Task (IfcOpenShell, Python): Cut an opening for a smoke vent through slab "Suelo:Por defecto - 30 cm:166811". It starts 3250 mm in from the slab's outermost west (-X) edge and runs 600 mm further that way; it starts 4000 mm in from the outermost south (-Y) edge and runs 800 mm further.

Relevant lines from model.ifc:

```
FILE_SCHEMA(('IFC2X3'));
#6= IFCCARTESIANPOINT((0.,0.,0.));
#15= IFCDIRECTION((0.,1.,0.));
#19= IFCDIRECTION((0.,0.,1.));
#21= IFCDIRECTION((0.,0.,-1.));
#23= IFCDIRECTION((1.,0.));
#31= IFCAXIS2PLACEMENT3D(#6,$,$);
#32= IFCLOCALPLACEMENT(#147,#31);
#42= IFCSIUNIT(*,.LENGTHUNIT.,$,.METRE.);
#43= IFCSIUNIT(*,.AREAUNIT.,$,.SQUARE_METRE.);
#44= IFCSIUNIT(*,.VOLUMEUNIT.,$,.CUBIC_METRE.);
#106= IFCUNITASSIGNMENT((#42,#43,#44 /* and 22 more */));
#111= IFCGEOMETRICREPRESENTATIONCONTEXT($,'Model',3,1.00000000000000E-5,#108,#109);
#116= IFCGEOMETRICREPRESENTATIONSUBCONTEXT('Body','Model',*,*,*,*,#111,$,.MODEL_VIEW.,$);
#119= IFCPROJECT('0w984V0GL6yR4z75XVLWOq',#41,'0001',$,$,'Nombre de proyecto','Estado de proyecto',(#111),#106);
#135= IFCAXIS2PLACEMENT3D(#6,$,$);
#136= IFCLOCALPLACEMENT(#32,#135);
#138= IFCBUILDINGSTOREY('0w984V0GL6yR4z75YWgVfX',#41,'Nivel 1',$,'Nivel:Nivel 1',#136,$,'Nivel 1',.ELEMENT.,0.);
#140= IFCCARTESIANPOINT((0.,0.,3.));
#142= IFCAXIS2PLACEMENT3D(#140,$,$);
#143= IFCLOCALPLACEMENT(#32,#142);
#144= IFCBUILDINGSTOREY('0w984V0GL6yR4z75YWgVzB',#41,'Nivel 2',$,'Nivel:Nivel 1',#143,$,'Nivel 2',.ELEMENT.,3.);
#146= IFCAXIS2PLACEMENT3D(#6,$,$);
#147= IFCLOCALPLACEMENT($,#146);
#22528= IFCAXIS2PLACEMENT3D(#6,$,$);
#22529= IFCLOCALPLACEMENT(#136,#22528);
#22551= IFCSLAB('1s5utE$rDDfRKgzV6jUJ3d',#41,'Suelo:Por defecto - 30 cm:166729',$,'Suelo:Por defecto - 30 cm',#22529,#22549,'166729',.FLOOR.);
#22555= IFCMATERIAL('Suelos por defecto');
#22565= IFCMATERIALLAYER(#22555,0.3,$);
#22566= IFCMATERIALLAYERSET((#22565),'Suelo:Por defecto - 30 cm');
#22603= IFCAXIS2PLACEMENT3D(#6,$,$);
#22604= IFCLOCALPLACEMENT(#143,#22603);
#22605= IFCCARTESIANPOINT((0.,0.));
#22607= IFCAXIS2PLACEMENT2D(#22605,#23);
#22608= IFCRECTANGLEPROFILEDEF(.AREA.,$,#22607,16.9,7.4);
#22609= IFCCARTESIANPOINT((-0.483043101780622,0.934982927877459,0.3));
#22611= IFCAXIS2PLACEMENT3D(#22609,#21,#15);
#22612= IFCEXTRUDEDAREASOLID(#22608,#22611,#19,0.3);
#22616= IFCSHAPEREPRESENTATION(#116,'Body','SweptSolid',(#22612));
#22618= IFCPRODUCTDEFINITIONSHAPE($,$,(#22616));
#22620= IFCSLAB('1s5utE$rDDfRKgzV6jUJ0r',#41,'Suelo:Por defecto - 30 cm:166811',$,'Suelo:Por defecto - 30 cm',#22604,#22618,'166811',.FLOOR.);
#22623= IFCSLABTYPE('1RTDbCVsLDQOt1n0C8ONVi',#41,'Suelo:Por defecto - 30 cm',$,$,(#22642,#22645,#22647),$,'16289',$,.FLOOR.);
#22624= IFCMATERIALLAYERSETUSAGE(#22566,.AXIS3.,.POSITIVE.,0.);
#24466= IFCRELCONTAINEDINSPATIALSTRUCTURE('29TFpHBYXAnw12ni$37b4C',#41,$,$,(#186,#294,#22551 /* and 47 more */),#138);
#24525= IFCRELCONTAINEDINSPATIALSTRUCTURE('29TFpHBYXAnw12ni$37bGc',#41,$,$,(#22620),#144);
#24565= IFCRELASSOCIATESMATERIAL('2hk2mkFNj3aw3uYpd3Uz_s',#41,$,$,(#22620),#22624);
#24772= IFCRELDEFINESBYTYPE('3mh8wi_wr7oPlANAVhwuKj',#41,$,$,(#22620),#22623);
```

```python
import numpy as np
import ifcopenshell
import ifcopenshell.api.feature
import ifcopenshell.api.geometry
import ifcopenshell.api.root
import ifcopenshell.geom
import ifcopenshell.util.placement
import ifcopenshell.util.representation
import ifcopenshell.util.shape
import ifcopenshell.util.unit

model = ifcopenshell.open("model.ifc")
unit_scale = ifcopenshell.util.unit.calculate_unit_scale(model)
settings = ifcopenshell.geom.settings()


def volume(element):
    """Net volume in cubic metres, openings subtracted."""
    shape = ifcopenshell.geom.create_shape(settings, element)
    return ifcopenshell.util.shape.get_volume(shape.geometry)


slab = model.by_guid("1s5utE$rDDfRKgzV6jUJ0r")
before = volume(slab)

# Extent in the slab's own axes, in metres. The edges named are its -X and -Y sides.
slab_shape = ifcopenshell.geom.create_shape(settings, slab)
vertices = ifcopenshell.util.shape.get_vertices(slab_shape.geometry)
x_min, y_min, bottom = vertices.min(axis=0)
top = vertices[:, 2].max()

opening = ifcopenshell.api.root.create_entity(model, ifc_class="IfcOpeningElement", name="Smoke vent opening")
context = ifcopenshell.util.representation.get_context(model, "Model", "Body", "MODEL_VIEW")
width, depth = 0.6, 0.8
outline = [(0.0, 0.0), (width, 0.0), (width, depth), (0.0, depth), (0.0, 0.0)]
# Overshoot both faces by 50 mm so the cut is clean.
shape = ifcopenshell.api.geometry.add_slab_representation(
    model, context=context, depth=top - bottom + 0.1, polyline=outline
)
ifcopenshell.api.geometry.assign_representation(model, product=opening, representation=shape)

matrix = ifcopenshell.util.placement.get_local_placement(slab.ObjectPlacement)
matrix[:, 3] = matrix @ np.append(np.array([x_min + 3.25, y_min + 4, bottom - 0.05]) / unit_scale, 1.0)
ifcopenshell.api.geometry.edit_object_placement(model, product=opening, matrix=matrix, is_si=False)
ifcopenshell.api.feature.add_feature(model, feature=opening, element=slab)

after = volume(slab)

print(f"slab volume {before:.3f} -> {after:.3f} m3")

model.write("model_v2.ifc")
```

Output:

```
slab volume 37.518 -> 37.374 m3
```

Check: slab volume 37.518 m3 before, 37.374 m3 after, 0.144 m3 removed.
